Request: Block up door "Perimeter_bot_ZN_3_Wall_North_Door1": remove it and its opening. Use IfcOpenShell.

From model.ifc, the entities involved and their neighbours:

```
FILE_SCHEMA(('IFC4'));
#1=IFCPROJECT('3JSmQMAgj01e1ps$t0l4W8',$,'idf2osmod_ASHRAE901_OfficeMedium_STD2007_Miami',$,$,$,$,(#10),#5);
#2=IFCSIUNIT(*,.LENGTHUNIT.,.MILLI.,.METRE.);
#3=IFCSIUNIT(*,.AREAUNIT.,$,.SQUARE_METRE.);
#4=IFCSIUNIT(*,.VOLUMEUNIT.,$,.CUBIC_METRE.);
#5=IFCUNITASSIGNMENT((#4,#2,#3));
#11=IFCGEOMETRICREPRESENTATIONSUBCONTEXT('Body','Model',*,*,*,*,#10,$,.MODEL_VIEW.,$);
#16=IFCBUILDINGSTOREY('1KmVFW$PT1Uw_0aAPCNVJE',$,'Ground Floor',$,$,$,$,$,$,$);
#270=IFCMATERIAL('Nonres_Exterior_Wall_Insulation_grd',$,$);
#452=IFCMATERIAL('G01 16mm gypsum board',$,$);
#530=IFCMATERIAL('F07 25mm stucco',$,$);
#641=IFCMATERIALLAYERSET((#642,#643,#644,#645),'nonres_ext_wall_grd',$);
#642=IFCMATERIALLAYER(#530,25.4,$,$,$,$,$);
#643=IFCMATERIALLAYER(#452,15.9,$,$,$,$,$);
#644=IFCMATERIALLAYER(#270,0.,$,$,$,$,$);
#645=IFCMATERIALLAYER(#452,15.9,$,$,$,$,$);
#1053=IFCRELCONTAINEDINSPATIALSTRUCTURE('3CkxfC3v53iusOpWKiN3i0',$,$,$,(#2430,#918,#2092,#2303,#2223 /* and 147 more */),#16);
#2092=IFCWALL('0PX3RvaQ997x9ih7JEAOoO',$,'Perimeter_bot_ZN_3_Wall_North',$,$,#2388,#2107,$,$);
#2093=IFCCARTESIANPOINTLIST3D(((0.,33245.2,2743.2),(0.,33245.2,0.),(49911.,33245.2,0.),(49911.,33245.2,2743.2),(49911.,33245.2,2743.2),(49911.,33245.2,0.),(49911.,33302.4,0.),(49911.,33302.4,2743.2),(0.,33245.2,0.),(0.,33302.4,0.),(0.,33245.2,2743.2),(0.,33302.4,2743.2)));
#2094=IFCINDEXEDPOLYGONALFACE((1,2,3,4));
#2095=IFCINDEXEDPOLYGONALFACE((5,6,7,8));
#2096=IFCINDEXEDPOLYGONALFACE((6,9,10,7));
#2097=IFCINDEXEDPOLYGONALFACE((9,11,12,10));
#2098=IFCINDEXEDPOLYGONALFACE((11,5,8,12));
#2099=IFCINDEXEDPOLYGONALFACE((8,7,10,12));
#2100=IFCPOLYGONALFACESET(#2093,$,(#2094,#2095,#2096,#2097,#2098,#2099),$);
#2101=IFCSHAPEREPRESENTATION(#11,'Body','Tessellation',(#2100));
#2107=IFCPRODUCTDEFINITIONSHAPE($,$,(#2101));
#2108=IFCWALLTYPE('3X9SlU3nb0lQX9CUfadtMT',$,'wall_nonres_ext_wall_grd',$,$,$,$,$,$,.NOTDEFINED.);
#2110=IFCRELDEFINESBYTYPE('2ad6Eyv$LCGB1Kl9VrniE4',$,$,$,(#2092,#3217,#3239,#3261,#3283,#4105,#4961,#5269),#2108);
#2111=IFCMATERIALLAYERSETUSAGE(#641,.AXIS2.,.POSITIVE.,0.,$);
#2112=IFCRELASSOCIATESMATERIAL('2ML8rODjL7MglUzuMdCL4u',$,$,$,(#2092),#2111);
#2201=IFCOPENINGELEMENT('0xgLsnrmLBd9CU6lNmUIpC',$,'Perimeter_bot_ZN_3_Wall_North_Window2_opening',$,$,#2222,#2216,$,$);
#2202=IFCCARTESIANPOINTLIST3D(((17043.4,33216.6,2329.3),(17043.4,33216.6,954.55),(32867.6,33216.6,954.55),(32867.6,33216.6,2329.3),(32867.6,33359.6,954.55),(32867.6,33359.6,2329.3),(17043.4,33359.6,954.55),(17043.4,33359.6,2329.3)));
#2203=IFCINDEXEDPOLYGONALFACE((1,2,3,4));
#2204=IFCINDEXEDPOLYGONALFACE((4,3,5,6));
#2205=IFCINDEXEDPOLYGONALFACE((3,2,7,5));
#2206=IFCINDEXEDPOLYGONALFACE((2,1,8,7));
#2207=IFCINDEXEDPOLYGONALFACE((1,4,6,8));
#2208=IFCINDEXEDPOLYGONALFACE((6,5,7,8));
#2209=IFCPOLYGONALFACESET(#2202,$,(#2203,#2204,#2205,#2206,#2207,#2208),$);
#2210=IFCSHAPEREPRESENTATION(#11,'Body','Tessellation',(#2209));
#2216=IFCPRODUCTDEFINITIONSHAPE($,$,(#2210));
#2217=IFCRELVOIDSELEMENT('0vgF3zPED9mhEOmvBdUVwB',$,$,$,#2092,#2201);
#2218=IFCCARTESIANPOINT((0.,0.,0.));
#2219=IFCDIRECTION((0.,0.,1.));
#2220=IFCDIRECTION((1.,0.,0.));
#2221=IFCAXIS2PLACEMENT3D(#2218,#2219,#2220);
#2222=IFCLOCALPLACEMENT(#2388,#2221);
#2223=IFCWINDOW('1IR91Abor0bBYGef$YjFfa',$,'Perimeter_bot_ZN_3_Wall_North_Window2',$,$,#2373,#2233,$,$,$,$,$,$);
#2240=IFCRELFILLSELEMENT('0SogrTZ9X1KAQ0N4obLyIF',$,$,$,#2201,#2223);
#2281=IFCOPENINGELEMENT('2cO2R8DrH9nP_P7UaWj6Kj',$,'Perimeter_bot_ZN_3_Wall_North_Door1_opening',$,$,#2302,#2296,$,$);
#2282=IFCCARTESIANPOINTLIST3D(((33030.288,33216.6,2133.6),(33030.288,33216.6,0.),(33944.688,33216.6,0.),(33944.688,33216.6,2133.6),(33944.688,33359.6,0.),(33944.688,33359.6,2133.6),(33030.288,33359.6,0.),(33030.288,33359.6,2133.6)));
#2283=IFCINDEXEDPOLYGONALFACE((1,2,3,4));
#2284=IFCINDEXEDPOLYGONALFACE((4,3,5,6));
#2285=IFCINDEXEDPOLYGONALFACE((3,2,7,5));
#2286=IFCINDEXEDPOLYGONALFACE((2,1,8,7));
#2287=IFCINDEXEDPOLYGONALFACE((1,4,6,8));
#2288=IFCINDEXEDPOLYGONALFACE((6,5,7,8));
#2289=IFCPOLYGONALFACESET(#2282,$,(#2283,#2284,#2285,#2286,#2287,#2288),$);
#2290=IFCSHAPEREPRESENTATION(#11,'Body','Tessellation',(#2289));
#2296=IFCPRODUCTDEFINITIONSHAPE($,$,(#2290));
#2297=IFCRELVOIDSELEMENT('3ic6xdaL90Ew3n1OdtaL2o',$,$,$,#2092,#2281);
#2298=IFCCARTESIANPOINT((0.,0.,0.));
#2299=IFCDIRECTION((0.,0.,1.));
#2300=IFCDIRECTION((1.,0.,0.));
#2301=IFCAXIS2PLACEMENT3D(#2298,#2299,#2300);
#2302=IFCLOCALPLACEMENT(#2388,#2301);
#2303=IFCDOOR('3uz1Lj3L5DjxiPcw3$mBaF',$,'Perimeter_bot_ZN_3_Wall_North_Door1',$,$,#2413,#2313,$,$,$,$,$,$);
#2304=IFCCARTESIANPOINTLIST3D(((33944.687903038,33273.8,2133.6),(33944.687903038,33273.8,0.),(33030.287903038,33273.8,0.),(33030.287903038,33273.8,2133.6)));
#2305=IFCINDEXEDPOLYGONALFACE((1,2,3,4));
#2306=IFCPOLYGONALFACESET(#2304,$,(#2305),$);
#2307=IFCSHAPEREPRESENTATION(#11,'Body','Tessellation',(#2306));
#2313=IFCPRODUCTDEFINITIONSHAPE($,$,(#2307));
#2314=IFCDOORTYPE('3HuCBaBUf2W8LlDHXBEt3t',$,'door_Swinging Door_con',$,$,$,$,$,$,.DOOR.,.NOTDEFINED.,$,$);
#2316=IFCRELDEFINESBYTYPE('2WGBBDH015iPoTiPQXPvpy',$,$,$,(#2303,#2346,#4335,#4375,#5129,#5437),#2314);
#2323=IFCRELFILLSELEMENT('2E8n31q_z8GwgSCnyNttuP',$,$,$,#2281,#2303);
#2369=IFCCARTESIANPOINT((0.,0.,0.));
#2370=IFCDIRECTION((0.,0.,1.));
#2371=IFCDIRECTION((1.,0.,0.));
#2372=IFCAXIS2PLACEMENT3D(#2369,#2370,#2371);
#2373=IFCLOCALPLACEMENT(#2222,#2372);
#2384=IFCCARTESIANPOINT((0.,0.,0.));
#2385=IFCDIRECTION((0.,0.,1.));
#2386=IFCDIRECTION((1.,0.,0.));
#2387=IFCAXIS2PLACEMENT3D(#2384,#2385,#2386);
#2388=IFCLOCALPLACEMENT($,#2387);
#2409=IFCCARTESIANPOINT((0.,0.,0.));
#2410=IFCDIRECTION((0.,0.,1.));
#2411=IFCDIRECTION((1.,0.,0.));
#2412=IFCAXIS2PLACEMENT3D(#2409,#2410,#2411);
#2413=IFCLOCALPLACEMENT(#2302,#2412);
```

```python
import ifcopenshell
import ifcopenshell.api.feature
import ifcopenshell.api.root
import ifcopenshell.geom
import ifcopenshell.util.shape

model = ifcopenshell.open("model.ifc")
settings = ifcopenshell.geom.settings()


def volume(element):
    """Net volume in cubic metres, openings subtracted."""
    shape = ifcopenshell.geom.create_shape(settings, element)
    return ifcopenshell.util.shape.get_volume(shape.geometry)


door = model.by_guid("3uz1Lj3L5DjxiPcw3$mBaF")
opening = door.FillsVoids[0].RelatingOpeningElement
wall = opening.VoidsElements[0].RelatingBuildingElement
before = volume(wall)

ifcopenshell.api.root.remove_product(model, product=door)
ifcopenshell.api.feature.remove_feature(model, feature=opening)

after = volume(wall)

print(f"wall volume {before:.3f} -> {after:.3f} m3")

model.write("model_edited.ifc")
```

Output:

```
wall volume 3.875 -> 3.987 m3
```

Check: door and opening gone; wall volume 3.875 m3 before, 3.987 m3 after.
